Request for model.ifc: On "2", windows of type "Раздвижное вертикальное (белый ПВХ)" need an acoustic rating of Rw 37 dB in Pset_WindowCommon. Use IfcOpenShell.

First a look at what the model holds.

```python
import ifcopenshell
import ifcopenshell.util.element

model = ifcopenshell.open("model.ifc")
print(model.schema)
storey = next(s for s in model.by_type("IfcBuildingStorey") if s.Name == "2")
windows = [e for e in ifcopenshell.util.element.get_decomposition(storey) if e.is_a("IfcWindow")]
seen = {}
for e in windows:
    element_type = ifcopenshell.util.element.get_type(e)
    key = (element_type.Name if element_type != e and element_type else None, ifcopenshell.util.element.get_pset(e, "Pset_WindowCommon", "AcousticRating"))
    seen[key] = seen.get(key, 0) + 1
for (name, value), count in sorted(seen.items(), key=str):
    print(count, "x", name, "|", value)
```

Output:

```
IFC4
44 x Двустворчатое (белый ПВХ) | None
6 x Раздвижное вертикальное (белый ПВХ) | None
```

```python
import ifcopenshell
import ifcopenshell.api.pset
import ifcopenshell.util.element

model = ifcopenshell.open("model.ifc")

storey = next(s for s in model.by_type("IfcBuildingStorey") if s.Name == "2")
windows = [e for e in ifcopenshell.util.element.get_decomposition(storey) if e.is_a("IfcWindow")]

count = 0
for e in windows:
    element_type = ifcopenshell.util.element.get_type(e)
    if element_type in (None, e) or element_type.Name != "Раздвижное вертикальное (белый ПВХ)":
        continue
    # add_pset returns the element's existing set when there is one.
    pset = ifcopenshell.api.pset.add_pset(model, product=e, name="Pset_WindowCommon")
    ifcopenshell.api.pset.edit_pset(model, pset=pset, properties={"AcousticRating": "Rw 37 dB"})
    count += 1

print(count, "windows updated")

model.write("model_rev.ifc")
```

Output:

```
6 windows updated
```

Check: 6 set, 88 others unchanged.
